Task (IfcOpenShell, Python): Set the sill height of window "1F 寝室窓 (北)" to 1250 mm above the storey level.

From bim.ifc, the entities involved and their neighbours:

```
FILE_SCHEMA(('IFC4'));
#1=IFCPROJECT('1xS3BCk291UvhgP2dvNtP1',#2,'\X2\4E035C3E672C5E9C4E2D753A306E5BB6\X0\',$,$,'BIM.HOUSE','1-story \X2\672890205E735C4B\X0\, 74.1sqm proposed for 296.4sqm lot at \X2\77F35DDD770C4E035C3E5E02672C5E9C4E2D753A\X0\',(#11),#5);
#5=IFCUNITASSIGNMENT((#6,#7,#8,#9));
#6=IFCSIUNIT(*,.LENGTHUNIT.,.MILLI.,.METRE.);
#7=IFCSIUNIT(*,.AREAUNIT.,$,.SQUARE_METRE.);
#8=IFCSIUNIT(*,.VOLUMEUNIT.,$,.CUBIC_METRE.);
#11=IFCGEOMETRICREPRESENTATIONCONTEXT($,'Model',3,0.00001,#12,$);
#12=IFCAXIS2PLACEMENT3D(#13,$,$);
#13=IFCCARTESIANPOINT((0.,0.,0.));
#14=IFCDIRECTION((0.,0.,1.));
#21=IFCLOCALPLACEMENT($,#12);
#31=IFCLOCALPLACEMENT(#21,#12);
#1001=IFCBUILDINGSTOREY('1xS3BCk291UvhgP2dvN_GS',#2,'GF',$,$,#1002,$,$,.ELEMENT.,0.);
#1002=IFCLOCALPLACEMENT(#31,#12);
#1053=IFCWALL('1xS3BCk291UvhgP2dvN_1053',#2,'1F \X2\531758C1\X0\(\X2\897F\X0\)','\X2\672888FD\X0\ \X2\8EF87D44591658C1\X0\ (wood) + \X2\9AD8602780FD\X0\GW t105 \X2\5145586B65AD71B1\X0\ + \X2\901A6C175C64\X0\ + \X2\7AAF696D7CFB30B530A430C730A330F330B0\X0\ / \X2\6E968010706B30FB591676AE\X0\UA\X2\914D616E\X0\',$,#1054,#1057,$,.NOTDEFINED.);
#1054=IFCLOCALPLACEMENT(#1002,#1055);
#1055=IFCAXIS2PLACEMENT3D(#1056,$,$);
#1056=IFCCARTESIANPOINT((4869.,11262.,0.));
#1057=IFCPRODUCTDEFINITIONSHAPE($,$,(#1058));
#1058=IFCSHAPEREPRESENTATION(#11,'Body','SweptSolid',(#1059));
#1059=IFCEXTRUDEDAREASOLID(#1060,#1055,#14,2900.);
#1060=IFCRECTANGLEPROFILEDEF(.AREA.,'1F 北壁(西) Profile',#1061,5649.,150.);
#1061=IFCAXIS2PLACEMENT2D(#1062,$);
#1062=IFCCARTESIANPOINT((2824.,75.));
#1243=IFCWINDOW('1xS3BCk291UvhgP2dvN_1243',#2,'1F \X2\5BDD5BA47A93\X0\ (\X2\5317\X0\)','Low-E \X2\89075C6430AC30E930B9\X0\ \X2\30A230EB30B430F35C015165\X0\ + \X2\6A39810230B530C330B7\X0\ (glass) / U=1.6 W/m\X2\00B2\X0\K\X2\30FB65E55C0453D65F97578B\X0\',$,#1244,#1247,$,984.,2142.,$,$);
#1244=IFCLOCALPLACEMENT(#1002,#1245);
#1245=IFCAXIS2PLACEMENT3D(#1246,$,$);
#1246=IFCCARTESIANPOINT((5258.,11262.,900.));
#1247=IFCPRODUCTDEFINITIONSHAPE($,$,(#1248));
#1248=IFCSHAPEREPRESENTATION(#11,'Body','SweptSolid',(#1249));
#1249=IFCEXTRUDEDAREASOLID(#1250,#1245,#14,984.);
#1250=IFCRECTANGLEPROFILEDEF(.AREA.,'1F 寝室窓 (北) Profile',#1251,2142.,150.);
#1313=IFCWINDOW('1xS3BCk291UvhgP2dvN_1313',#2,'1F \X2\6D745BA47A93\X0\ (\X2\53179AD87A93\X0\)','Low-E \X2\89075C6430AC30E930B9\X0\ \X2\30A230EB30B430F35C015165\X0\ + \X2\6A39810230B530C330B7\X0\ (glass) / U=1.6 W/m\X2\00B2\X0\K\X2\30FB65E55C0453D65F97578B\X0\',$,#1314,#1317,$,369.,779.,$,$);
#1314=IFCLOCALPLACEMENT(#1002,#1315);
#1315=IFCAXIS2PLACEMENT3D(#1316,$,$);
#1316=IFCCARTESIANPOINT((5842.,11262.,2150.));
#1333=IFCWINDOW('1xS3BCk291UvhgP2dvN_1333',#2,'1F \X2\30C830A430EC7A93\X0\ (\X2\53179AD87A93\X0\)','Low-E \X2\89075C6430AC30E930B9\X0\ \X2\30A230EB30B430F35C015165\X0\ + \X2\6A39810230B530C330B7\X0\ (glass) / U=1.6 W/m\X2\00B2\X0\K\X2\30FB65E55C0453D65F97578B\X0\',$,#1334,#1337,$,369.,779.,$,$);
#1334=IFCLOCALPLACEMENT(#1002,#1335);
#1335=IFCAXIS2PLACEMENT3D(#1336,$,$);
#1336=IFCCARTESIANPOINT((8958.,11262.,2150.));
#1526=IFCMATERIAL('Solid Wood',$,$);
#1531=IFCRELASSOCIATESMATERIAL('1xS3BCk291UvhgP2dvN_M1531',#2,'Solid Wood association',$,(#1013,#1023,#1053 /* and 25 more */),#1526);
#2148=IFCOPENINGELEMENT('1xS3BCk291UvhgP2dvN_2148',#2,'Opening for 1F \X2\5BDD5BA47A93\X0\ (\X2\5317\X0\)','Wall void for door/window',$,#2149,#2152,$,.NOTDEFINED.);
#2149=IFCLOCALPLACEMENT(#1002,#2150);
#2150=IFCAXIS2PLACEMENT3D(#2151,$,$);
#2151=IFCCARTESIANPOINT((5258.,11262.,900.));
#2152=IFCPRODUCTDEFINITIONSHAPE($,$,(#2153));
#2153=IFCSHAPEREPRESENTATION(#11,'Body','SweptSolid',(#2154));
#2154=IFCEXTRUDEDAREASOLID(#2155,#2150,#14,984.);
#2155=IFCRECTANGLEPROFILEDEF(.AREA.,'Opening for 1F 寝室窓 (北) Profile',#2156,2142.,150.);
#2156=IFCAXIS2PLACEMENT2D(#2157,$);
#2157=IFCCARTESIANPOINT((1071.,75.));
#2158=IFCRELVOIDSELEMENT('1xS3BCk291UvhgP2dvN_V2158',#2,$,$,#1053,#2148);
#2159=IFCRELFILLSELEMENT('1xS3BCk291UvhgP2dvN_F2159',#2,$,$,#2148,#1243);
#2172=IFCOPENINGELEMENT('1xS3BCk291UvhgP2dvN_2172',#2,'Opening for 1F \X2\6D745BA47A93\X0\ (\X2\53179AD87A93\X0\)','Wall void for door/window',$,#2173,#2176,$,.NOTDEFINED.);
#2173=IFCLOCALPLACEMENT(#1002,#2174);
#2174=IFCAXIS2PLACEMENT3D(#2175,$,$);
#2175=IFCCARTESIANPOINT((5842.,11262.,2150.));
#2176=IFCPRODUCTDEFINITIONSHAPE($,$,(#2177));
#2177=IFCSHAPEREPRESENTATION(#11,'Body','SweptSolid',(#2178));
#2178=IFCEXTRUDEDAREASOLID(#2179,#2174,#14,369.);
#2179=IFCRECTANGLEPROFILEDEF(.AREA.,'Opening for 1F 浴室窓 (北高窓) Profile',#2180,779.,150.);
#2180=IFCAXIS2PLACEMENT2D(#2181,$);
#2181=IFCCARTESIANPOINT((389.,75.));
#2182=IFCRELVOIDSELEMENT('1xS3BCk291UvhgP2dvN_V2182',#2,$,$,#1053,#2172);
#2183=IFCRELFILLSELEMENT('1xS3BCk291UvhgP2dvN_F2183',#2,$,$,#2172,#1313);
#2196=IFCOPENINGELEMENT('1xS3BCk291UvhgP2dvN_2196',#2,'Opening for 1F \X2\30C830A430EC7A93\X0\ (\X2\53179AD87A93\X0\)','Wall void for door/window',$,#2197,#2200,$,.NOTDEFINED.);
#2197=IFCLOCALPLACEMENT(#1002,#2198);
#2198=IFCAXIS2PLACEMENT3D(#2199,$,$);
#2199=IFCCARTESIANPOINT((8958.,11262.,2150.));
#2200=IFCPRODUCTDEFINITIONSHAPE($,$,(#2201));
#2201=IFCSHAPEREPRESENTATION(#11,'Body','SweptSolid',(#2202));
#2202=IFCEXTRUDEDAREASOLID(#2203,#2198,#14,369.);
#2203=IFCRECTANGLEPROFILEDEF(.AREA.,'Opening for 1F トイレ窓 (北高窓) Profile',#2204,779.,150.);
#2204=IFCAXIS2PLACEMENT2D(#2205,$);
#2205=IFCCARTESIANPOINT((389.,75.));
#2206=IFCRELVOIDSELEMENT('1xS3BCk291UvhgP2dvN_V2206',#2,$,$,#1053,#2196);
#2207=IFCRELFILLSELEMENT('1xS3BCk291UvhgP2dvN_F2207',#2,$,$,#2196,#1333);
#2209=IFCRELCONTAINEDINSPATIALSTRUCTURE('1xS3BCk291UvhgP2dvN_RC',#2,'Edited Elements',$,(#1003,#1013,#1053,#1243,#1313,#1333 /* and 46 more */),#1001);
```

```python
import numpy as np
import ifcopenshell
import ifcopenshell.api.geometry
import ifcopenshell.geom
import ifcopenshell.util.element
import ifcopenshell.util.placement
import ifcopenshell.util.shape
import ifcopenshell.util.unit

model = ifcopenshell.open("bim.ifc")
unit_scale = ifcopenshell.util.unit.calculate_unit_scale(model)

window = model.by_guid("1xS3BCk291UvhgP2dvN_1243")
opening = window.FillsVoids[0].RelatingOpeningElement
storey = ifcopenshell.util.element.get_container(window, ifc_class="IfcBuildingStorey")
level = ifcopenshell.util.placement.get_local_placement(storey.ObjectPlacement)[2, 3]

# The opening's origin need not be at the sill, so measure its lowest point.
shape = ifcopenshell.geom.create_shape(ifcopenshell.geom.settings(), opening)
bottom = ifcopenshell.util.shape.get_shape_bottom_elevation(shape, shape.geometry) / unit_scale
dz = level + 1.25 / unit_scale - bottom

shift = np.array([0.0, 0.0, dz])
# The window is not placed relative to its opening, so move both.
for product in (opening, window):
    matrix = ifcopenshell.util.placement.get_local_placement(product.ObjectPlacement)
    matrix[:3, 3] += shift
    ifcopenshell.api.geometry.edit_object_placement(model, product=product, matrix=matrix, is_si=False)

print(f"moved by {dz * unit_scale:+.3f} m")

model.write("bim_v2.ifc")
```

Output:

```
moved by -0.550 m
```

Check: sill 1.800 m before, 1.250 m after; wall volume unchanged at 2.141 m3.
